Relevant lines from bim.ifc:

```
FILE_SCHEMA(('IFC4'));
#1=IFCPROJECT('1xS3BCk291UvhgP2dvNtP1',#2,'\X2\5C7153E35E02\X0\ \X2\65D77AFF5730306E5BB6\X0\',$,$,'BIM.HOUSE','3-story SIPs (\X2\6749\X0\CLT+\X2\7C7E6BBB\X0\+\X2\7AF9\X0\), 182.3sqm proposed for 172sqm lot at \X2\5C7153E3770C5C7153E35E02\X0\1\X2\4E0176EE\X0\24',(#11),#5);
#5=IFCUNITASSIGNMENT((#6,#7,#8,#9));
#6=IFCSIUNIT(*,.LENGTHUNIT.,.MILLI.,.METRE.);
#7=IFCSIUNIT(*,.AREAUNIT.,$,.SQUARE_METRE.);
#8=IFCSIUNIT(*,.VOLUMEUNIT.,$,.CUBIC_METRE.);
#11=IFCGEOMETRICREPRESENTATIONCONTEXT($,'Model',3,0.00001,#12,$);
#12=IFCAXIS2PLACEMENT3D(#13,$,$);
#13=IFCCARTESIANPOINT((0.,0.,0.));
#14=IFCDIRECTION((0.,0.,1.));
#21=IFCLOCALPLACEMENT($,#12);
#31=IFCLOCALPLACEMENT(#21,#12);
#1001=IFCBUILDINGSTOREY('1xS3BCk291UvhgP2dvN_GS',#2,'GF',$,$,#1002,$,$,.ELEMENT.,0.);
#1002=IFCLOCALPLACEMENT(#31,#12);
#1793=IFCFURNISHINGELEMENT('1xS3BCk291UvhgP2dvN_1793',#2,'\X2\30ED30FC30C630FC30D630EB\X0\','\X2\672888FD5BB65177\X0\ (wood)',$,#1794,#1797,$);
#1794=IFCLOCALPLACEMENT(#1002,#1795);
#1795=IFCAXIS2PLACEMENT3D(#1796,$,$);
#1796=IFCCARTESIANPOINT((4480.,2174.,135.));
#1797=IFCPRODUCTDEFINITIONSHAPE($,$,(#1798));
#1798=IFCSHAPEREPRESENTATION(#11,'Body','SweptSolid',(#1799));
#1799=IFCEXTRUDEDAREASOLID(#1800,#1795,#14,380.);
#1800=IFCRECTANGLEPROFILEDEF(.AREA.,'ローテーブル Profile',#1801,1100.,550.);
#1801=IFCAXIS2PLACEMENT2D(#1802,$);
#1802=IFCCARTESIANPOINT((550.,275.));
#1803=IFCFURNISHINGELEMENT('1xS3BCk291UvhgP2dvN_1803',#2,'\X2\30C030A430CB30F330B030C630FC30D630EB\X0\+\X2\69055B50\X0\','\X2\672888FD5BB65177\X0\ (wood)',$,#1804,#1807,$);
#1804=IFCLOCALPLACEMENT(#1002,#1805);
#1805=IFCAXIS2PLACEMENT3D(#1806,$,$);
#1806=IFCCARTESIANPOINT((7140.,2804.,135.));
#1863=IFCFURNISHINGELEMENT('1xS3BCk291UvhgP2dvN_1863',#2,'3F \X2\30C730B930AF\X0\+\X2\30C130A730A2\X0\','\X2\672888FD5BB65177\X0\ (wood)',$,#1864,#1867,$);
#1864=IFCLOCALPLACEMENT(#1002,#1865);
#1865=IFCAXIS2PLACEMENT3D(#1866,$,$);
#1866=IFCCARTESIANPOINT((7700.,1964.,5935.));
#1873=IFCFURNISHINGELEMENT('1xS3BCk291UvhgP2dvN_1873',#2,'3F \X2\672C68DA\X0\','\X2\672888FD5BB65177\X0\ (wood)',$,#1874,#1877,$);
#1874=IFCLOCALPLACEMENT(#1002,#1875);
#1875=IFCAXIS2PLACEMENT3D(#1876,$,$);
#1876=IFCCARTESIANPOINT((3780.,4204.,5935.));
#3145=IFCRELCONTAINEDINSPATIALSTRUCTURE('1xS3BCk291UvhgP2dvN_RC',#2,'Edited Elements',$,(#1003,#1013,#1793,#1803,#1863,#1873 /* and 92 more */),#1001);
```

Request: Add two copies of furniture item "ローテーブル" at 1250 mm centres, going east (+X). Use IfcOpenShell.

```python
import numpy as np
import ifcopenshell
import ifcopenshell.api.geometry
import ifcopenshell.api.root
import ifcopenshell.util.element
import ifcopenshell.util.placement
import ifcopenshell.util.unit

model = ifcopenshell.open("bim.ifc")
unit_scale = ifcopenshell.util.unit.calculate_unit_scale(model)


def reuse_history(source, copy):
    """copy_class also copies each property set's owner history, people and application; keep the originals."""
    for rel in copy.IsDefinedBy:
        if rel.is_a("IfcRelDefinesByProperties") and (history := rel.RelatingPropertyDefinition.OwnerHistory):
            rel.RelatingPropertyDefinition.OwnerHistory = source.OwnerHistory
            ifcopenshell.util.element.remove_deep2(model, history)


source = model.by_guid("1xS3BCk291UvhgP2dvN_1793")
base = ifcopenshell.util.placement.get_local_placement(source.ObjectPlacement)
step = np.array([1.0, 0.0, 0.0]) * 1.25 / unit_scale

for i in range(1, 3):
    copy = ifcopenshell.api.root.copy_class(model, product=source)
    copy.Representation = ifcopenshell.util.element.copy_deep(
        model, source.Representation, exclude=["IfcGeometricRepresentationContext", "IfcRepresentationMap"]
    )
    reuse_history(source, copy)
    matrix = base.copy()
    matrix[:3, 3] += i * step
    print("added at", matrix[:3, 3].round(3) + 0.0)
    ifcopenshell.api.geometry.edit_object_placement(model, product=copy, matrix=matrix, is_si=False)

model.write("bim_updated.ifc")
```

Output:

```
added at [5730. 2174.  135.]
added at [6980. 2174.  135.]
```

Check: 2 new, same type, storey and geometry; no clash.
